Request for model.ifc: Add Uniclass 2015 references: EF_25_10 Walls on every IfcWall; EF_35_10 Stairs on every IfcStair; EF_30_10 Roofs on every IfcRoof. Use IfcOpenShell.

First a look at what the model holds.

```python
import ifcopenshell

model = ifcopenshell.open("model.ifc")
print(model.schema)
print("classifications:", [c.Name for c in model.by_type("IfcClassification")])
for ifc_class in ("IfcDoor", "IfcRoof", "IfcStair", "IfcWall", "IfcWindow"):
    print(ifc_class, len(model.by_type(ifc_class)))
```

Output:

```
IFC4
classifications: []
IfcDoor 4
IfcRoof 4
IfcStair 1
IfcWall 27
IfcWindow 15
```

```python
import ifcopenshell
import ifcopenshell.api.classification

model = ifcopenshell.open("model.ifc")

system = ifcopenshell.api.classification.add_classification(model, classification="Uniclass 2015")

codes = {
    "IfcWall": ("EF_25_10", "Walls"),
    "IfcStair": ("EF_35_10", "Stairs"),
    "IfcRoof": ("EF_30_10", "Roofs"),
}
for ifc_class, (code, name) in codes.items():
    products = model.by_type(ifc_class)
    ifcopenshell.api.classification.add_reference(
        model, products=products, classification=system, identification=code, name=name
    )
    print(code, len(products))

model.write("model_updated.ifc")
```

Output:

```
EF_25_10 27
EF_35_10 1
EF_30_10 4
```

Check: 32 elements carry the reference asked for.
